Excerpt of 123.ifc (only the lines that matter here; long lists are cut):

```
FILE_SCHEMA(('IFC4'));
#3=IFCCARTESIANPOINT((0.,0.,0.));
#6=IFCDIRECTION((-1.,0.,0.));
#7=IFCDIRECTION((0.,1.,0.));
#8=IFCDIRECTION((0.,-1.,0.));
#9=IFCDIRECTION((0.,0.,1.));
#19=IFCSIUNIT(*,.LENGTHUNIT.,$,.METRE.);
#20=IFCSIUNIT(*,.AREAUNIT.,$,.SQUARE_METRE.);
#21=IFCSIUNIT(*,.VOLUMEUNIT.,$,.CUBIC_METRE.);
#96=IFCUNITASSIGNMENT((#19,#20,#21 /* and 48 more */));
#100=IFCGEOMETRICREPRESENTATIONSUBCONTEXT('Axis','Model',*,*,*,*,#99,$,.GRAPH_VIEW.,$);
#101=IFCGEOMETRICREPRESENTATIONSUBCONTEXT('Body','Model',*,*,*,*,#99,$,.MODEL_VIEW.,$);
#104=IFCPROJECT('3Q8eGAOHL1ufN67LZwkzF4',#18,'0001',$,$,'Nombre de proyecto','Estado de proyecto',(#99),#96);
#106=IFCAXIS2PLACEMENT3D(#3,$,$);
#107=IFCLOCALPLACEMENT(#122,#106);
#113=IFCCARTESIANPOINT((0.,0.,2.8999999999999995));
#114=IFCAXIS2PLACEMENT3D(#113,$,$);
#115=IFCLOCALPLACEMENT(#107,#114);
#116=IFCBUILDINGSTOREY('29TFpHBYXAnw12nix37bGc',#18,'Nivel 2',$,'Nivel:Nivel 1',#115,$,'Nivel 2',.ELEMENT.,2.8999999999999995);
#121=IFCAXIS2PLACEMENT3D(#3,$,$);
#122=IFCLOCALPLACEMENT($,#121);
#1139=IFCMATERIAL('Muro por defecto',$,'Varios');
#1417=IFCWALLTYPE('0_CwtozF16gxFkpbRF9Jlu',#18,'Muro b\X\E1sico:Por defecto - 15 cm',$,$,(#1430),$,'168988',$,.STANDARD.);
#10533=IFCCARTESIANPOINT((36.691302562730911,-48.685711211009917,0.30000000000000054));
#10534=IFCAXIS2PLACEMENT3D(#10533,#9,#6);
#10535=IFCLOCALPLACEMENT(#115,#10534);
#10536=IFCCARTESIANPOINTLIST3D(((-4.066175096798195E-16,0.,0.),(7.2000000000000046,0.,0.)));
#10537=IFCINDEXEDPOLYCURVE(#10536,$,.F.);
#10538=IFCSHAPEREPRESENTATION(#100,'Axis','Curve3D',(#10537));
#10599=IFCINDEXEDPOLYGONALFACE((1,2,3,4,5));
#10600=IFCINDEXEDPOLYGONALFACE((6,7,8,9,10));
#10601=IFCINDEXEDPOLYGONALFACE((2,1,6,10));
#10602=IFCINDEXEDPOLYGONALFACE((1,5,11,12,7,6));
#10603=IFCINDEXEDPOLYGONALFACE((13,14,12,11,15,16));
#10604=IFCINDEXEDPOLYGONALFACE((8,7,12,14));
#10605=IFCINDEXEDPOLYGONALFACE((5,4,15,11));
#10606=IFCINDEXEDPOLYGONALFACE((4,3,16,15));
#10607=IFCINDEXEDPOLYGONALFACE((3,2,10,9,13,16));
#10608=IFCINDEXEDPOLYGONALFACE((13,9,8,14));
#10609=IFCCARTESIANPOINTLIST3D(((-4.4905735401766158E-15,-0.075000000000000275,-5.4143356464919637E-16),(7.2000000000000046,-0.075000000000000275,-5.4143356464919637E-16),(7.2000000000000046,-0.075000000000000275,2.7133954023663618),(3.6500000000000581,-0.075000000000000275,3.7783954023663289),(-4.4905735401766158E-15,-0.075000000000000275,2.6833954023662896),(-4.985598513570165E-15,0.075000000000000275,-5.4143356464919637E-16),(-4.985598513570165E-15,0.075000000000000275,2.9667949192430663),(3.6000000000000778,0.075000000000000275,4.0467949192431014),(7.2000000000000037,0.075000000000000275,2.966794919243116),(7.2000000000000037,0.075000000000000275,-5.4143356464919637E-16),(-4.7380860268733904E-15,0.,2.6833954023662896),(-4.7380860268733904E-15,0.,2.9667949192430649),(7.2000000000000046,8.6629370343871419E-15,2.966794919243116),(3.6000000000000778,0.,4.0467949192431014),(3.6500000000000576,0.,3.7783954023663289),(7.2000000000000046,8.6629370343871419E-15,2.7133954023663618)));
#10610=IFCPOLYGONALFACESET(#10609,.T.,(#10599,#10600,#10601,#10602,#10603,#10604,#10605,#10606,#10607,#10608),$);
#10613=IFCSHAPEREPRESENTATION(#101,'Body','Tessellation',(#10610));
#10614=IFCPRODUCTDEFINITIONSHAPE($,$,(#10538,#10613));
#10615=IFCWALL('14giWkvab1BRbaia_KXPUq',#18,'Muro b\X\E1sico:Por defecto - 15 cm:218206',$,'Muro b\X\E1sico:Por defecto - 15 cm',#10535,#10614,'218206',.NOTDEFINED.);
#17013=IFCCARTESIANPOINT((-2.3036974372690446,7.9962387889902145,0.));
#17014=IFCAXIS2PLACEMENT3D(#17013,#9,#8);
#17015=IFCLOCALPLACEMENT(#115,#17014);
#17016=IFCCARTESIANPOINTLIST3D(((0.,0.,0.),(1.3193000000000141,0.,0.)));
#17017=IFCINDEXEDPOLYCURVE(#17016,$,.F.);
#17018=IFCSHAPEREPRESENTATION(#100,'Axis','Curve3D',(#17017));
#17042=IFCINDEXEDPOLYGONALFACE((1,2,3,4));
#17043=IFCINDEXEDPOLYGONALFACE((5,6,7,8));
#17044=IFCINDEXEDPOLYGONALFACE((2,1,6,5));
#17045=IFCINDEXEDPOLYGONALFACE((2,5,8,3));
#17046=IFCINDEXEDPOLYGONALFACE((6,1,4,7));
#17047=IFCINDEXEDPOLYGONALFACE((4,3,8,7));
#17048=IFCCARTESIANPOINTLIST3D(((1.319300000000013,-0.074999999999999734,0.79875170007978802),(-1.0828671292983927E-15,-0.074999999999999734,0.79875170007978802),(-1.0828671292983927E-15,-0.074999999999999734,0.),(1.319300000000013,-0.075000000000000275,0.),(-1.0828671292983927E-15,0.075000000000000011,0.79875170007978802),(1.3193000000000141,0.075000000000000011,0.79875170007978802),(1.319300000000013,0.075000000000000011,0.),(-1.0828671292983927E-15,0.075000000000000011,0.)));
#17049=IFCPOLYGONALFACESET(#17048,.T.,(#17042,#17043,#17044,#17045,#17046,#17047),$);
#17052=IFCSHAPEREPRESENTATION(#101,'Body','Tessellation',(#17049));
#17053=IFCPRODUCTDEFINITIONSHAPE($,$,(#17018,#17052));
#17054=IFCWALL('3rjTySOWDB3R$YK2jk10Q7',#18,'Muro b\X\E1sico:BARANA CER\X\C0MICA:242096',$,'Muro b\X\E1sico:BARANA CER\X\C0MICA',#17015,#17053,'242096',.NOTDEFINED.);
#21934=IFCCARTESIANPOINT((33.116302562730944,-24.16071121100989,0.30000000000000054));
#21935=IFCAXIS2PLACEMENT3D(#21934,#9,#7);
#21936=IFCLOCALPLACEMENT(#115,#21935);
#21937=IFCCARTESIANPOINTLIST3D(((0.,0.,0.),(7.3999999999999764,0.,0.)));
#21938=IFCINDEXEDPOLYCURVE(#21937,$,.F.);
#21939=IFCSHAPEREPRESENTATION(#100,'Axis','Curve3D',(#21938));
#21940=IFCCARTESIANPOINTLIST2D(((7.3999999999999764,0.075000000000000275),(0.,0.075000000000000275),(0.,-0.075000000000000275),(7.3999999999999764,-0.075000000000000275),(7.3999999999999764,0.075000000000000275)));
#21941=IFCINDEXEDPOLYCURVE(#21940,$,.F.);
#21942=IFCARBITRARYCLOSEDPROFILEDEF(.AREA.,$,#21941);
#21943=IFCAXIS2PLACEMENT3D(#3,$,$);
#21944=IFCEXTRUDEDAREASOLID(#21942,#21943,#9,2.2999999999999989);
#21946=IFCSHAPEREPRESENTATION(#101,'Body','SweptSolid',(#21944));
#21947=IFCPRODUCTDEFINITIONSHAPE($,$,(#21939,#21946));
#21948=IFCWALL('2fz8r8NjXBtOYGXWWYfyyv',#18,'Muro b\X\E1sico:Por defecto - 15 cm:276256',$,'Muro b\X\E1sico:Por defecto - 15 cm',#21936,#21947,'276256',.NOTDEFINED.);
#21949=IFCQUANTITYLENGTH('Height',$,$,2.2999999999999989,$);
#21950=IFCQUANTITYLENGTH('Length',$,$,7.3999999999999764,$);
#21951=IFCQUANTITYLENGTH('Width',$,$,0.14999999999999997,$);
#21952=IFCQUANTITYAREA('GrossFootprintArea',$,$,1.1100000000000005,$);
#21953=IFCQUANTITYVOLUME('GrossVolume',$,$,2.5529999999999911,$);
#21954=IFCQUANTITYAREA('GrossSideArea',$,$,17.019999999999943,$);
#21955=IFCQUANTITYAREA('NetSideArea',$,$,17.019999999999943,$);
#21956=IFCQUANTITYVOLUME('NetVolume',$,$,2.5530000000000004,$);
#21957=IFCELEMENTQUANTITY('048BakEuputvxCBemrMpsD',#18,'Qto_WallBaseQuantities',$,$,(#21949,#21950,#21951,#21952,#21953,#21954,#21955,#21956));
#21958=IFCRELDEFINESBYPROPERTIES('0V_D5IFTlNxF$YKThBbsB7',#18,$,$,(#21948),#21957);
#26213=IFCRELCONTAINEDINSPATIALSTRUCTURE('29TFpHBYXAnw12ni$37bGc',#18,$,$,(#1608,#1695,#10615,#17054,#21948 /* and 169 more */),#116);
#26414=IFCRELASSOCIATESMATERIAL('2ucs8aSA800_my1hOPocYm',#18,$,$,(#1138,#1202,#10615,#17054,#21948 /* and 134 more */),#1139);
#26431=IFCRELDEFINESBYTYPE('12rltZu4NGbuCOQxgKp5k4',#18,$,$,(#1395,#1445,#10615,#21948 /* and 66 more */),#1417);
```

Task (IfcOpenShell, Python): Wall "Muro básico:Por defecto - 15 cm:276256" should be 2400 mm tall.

```python
import ifcopenshell
import ifcopenshell.api.pset
import ifcopenshell.geom
import ifcopenshell.util.element
import ifcopenshell.util.representation
import ifcopenshell.util.shape
import ifcopenshell.util.unit

model = ifcopenshell.open("123.ifc")
unit_scale = ifcopenshell.util.unit.calculate_unit_scale(model)
area_scale = ifcopenshell.util.unit.calculate_unit_scale(model, "AREAUNIT")
volume_scale = ifcopenshell.util.unit.calculate_unit_scale(model, "VOLUMEUNIT")
settings = ifcopenshell.geom.settings()


def volume(element):
    """Net volume in cubic metres, openings subtracted."""
    shape = ifcopenshell.geom.create_shape(settings, element)
    return ifcopenshell.util.shape.get_volume(shape.geometry)


wall = model.by_guid("2fz8r8NjXBtOYGXWWYfyyv")
before = volume(wall)

body = ifcopenshell.util.representation.get_representation(wall, "Model", "Body")
solid = body.Items[0]
old_height = solid.Depth
solid.Depth = 2.4 / unit_scale
after = volume(wall)
thickness = 0.15  # wall thickness in metres

# Update the stored height, areas and volumes.
qto = model.by_id(ifcopenshell.util.element.get_pset(wall, "Qto_WallBaseQuantities", should_inherit=False)["id"])
ifcopenshell.api.pset.edit_qto(model, qto=qto, properties={
    "Height": solid.Depth,
    "GrossVolume": ifcopenshell.util.element.get_pset(wall, "Qto_WallBaseQuantities", "GrossVolume") * solid.Depth / old_height,
    "GrossSideArea": ifcopenshell.util.element.get_pset(wall, "Qto_WallBaseQuantities", "GrossSideArea") * solid.Depth / old_height,
    "NetSideArea": after / thickness / area_scale,
    "NetVolume": after / volume_scale,
})

print(f"height {old_height:g} -> {solid.Depth:g}, volume {before:.3f} -> {after:.3f} m3")

model.write("123_rev.ifc")
```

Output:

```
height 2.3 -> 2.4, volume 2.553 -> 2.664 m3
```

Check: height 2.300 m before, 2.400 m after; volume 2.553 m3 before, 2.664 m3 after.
